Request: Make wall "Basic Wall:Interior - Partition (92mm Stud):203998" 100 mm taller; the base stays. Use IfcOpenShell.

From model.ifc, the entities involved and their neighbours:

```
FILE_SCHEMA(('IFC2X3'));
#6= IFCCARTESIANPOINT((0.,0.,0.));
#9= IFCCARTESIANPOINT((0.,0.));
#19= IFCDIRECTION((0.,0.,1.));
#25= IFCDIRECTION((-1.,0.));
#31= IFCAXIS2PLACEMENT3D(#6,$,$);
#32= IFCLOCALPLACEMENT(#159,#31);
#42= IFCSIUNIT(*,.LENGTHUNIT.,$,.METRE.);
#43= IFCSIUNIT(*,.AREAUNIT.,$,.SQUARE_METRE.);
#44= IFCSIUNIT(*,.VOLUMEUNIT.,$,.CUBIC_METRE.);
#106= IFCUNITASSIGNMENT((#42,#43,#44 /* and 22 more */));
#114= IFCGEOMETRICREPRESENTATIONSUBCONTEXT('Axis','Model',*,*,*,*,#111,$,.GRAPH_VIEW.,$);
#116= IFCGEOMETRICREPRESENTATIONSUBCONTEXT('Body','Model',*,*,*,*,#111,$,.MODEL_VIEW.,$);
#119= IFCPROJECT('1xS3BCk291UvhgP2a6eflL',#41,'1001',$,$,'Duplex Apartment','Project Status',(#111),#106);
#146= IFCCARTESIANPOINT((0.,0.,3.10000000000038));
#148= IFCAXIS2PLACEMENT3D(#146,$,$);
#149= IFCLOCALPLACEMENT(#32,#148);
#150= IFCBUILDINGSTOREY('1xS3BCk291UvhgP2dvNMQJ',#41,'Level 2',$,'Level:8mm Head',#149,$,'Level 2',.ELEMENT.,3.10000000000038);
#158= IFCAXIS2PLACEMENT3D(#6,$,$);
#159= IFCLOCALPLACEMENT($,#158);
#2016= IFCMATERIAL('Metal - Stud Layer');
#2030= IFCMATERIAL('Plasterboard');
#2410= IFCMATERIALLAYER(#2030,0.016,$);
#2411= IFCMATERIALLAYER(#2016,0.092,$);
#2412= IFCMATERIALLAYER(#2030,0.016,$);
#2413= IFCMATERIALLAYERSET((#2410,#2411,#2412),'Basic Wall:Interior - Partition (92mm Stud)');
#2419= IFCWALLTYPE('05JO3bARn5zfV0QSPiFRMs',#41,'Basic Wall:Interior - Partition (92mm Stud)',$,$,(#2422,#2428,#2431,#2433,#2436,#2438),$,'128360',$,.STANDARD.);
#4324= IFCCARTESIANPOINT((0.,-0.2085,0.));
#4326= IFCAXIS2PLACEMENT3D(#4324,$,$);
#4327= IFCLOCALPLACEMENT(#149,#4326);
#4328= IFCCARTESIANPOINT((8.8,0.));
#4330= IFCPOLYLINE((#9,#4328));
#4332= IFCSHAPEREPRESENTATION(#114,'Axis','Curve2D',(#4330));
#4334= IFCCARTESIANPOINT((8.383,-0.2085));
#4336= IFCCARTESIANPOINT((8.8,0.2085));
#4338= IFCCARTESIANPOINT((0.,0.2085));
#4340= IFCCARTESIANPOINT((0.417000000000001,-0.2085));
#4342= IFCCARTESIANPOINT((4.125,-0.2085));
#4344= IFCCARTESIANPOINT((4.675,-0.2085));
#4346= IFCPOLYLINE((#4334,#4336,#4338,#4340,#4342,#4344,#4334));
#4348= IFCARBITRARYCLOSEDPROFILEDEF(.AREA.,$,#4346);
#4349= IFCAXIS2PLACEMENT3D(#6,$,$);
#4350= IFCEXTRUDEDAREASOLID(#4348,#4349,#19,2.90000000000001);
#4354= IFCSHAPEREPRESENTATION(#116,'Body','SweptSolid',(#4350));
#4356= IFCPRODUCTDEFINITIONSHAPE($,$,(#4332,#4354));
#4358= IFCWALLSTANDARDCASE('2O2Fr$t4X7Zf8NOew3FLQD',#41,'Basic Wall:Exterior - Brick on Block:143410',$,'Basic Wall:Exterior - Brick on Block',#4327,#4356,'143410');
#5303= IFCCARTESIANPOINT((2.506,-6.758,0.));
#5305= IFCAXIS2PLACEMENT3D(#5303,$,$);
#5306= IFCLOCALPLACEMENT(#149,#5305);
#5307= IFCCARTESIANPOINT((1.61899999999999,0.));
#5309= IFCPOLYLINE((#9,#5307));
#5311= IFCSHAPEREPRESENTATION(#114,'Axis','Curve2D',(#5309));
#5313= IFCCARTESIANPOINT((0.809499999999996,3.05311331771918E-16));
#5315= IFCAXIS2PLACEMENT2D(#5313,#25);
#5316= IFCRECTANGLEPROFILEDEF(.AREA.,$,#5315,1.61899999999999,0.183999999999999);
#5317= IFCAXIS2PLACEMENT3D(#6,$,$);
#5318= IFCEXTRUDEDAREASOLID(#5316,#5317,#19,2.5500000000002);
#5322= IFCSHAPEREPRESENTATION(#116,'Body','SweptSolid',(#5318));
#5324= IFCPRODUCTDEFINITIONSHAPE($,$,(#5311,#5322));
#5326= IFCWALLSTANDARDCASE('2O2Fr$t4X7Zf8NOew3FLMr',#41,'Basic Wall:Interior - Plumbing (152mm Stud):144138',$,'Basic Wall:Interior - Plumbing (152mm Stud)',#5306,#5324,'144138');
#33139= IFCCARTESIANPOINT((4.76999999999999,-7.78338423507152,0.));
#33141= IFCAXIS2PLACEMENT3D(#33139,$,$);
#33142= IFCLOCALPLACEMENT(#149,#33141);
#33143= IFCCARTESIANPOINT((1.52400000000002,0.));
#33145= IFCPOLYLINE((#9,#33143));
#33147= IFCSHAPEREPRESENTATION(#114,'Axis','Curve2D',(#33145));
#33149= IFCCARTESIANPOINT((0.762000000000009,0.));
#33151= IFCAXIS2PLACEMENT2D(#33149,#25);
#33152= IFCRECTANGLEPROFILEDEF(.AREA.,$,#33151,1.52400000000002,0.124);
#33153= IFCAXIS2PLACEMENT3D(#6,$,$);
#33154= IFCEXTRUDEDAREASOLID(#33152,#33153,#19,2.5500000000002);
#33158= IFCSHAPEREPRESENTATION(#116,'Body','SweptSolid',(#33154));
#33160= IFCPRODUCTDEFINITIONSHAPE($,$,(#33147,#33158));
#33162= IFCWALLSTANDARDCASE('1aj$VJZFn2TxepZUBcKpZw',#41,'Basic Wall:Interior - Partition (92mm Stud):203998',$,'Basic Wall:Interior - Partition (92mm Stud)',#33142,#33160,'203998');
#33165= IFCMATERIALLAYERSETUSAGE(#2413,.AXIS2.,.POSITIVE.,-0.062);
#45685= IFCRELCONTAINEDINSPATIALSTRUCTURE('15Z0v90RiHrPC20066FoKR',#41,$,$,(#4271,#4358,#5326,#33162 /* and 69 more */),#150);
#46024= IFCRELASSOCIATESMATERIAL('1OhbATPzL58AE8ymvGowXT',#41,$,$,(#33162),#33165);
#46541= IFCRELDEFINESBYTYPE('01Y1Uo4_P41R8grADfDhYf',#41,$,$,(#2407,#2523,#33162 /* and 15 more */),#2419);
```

```python
import ifcopenshell
import ifcopenshell.geom
import ifcopenshell.util.representation
import ifcopenshell.util.shape
import ifcopenshell.util.unit

model = ifcopenshell.open("model.ifc")
unit_scale = ifcopenshell.util.unit.calculate_unit_scale(model)
settings = ifcopenshell.geom.settings()


def volume(element):
    """Net volume in cubic metres, openings subtracted."""
    shape = ifcopenshell.geom.create_shape(settings, element)
    return ifcopenshell.util.shape.get_volume(shape.geometry)


wall = model.by_guid("1aj$VJZFn2TxepZUBcKpZw")
before = volume(wall)

body = ifcopenshell.util.representation.get_representation(wall, "Model", "Body")
solid = body.Items[0]
old_height = solid.Depth
solid.Depth += 0.1 / unit_scale
after = volume(wall)

print(f"height {old_height:g} -> {solid.Depth:g}, volume {before:.3f} -> {after:.3f} m3")

model.write("model_edited.ifc")
```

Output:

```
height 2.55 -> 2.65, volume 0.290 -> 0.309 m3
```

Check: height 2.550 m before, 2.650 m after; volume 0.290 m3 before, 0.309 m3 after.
